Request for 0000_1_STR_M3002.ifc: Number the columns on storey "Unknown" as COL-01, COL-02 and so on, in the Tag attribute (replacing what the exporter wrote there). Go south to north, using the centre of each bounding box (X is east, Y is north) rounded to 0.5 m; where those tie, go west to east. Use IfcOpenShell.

First a look at what the model holds.

```python
import ifcopenshell
import ifcopenshell.util.element
import ifcopenshell.util.placement

model = ifcopenshell.open("0000_1_STR_M3002.ifc")
print(model.schema)
storey = next(s for s in model.by_type("IfcBuildingStorey") if s.Name == "Unknown")
columns = [e for e in ifcopenshell.util.element.get_decomposition(storey) if e.is_a("IfcColumn")]
for e in sorted(columns, key=lambda e: e.id()):
    origin = ifcopenshell.util.placement.get_local_placement(e.ObjectPlacement)[:3, 3]
    print(e.id(), e.Tag, e.Name, origin.round(2) + 0.0, sep=" | ")
```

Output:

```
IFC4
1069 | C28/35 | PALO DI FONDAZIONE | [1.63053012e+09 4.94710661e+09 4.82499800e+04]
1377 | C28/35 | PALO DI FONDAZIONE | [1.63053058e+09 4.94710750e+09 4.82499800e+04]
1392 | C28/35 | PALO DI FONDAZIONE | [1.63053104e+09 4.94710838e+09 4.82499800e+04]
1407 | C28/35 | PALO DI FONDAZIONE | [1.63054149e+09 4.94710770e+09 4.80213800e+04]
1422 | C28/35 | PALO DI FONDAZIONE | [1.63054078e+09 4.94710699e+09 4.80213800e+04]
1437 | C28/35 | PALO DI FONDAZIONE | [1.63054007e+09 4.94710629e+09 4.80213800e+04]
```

```python
import ifcopenshell
import ifcopenshell.geom
import ifcopenshell.util.element
import ifcopenshell.util.shape

model = ifcopenshell.open("0000_1_STR_M3002.ifc")
settings = ifcopenshell.geom.settings()
settings.set("use-world-coords", True)


def centre(element):
    shape = ifcopenshell.geom.create_shape(settings, element)
    return ifcopenshell.util.shape.get_bbox_centroid(shape.geometry)


storey = next(s for s in model.by_type("IfcBuildingStorey") if s.Name == "Unknown")
columns = [e for e in ifcopenshell.util.element.get_decomposition(storey) if e.is_a("IfcColumn")]

# Insertion points can sit at a corner or the storey origin, so sort by the geometry (in metres).
centres = {e: centre(e) for e in columns}
columns.sort(key=lambda e: (round(centres[e][1] / 0.5), centres[e][0]))

for i, e in enumerate(columns, start=1):
    number = f"COL-{i:02d}"
    e.Tag = number
    print(e.id(), number)

model.write("0000_1_STR_M3002_edited.ifc")
```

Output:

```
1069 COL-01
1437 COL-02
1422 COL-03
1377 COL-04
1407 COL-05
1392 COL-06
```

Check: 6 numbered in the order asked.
